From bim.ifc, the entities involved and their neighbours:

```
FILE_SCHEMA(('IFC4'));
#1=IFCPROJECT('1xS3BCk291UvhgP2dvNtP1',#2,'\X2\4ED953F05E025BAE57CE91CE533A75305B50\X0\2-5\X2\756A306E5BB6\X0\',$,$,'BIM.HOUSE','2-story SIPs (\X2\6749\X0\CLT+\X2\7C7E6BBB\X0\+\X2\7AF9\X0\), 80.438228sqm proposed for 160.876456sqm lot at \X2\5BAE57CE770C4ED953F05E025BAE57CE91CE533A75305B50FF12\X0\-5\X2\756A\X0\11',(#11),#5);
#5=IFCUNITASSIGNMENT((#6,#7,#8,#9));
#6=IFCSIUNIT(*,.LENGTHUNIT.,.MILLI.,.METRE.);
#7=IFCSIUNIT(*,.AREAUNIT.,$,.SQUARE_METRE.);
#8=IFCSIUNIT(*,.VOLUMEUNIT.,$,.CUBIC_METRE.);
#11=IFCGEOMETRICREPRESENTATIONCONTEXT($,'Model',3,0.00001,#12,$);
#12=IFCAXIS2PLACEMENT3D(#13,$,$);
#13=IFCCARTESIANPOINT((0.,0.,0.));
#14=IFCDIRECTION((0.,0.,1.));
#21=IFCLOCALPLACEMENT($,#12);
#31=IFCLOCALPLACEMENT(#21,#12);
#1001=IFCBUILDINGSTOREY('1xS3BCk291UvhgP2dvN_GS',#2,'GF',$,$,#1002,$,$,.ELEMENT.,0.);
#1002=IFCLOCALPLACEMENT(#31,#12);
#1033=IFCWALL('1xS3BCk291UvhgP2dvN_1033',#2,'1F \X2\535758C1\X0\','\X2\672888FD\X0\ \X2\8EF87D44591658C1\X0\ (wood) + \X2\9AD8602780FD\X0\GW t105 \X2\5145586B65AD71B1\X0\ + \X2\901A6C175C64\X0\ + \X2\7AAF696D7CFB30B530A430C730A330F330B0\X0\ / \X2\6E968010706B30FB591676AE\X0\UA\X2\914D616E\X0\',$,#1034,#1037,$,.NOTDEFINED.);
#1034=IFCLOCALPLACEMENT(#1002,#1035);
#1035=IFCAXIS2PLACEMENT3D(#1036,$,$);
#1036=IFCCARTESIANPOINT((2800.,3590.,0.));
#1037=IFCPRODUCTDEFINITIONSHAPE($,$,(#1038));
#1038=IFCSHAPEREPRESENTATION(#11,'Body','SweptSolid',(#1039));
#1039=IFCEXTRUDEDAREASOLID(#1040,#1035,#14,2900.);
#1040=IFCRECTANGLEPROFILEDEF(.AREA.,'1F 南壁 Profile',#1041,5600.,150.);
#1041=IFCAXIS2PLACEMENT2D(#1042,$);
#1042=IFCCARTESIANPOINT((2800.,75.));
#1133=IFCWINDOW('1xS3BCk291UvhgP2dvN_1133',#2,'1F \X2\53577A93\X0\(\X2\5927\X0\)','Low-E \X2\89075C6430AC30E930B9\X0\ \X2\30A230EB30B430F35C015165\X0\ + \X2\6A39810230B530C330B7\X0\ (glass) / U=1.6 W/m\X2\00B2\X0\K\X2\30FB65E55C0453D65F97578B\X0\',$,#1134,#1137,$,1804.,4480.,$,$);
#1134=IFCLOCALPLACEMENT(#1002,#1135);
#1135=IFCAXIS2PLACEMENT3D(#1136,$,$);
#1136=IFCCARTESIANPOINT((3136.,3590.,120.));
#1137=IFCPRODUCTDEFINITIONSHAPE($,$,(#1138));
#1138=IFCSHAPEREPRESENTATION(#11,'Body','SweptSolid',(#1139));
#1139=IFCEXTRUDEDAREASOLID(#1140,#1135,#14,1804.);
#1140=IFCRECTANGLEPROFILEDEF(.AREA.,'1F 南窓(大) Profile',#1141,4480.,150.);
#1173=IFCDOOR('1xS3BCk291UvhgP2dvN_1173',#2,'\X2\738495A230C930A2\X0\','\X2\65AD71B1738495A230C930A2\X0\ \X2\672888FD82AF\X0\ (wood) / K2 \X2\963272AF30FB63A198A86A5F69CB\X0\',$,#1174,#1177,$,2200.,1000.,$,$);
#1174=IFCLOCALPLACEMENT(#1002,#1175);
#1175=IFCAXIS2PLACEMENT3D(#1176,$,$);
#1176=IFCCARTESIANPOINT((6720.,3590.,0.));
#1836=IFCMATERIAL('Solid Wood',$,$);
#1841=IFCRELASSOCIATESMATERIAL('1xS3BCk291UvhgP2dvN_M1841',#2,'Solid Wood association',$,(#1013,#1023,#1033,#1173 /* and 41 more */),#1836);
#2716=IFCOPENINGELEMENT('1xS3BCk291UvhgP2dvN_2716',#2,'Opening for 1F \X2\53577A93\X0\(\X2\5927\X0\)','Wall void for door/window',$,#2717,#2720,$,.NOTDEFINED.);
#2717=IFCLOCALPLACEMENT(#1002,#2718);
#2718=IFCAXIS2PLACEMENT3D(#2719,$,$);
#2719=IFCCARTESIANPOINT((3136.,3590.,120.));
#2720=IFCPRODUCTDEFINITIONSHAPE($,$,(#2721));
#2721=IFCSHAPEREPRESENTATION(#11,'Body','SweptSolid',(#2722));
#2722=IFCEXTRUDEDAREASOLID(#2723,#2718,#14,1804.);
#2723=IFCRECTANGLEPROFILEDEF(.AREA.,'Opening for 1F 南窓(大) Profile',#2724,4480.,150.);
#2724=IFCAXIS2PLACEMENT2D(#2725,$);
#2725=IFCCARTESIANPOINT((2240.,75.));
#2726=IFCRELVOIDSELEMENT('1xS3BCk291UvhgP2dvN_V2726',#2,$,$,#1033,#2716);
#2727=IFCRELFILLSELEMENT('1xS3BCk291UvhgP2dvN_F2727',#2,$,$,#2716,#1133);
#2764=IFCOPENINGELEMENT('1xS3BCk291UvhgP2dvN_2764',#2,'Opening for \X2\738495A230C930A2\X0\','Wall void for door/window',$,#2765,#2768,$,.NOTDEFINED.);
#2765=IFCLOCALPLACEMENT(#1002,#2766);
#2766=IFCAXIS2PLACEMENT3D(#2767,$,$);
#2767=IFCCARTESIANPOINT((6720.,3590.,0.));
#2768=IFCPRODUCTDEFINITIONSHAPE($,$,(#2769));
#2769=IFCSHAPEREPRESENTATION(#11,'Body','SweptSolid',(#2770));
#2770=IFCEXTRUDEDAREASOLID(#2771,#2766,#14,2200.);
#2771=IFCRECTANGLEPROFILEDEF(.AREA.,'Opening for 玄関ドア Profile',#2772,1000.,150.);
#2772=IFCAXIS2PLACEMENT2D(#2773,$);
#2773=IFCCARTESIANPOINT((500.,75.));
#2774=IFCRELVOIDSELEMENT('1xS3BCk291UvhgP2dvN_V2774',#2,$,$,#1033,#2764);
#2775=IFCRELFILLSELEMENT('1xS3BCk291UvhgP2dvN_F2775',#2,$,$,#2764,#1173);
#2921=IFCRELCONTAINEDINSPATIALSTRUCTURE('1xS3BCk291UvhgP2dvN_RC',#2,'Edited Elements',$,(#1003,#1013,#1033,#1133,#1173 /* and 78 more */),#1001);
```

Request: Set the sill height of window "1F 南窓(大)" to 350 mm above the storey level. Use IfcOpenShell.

```python
import numpy as np
import ifcopenshell
import ifcopenshell.api.geometry
import ifcopenshell.geom
import ifcopenshell.util.element
import ifcopenshell.util.placement
import ifcopenshell.util.shape
import ifcopenshell.util.unit

model = ifcopenshell.open("bim.ifc")
unit_scale = ifcopenshell.util.unit.calculate_unit_scale(model)

window = model.by_guid("1xS3BCk291UvhgP2dvN_1133")
opening = window.FillsVoids[0].RelatingOpeningElement
storey = ifcopenshell.util.element.get_container(window, ifc_class="IfcBuildingStorey")
level = ifcopenshell.util.placement.get_local_placement(storey.ObjectPlacement)[2, 3]

# The opening's origin need not be at the sill, so measure its lowest point.
shape = ifcopenshell.geom.create_shape(ifcopenshell.geom.settings(), opening)
bottom = ifcopenshell.util.shape.get_shape_bottom_elevation(shape, shape.geometry) / unit_scale
dz = level + 0.35 / unit_scale - bottom

shift = np.array([0.0, 0.0, dz])
# The window is not placed relative to its opening, so move both.
for product in (opening, window):
    matrix = ifcopenshell.util.placement.get_local_placement(product.ObjectPlacement)
    matrix[:3, 3] += shift
    ifcopenshell.api.geometry.edit_object_placement(model, product=product, matrix=matrix, is_si=False)

print(f"moved by {dz * unit_scale:+.3f} m")

model.write("bim_v2.ifc")
```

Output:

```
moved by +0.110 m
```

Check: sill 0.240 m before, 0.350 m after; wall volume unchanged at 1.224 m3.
